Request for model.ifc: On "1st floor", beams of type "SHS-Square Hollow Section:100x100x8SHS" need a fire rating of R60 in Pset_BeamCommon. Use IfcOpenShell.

First a look at what the model holds.

```python
import ifcopenshell
import ifcopenshell.util.element

model = ifcopenshell.open("model.ifc")
print(model.schema)
storey = next(s for s in model.by_type("IfcBuildingStorey") if s.Name == "1st floor")
beams = [e for e in ifcopenshell.util.element.get_decomposition(storey) if e.is_a("IfcBeam")]
seen = {}
for e in beams:
    element_type = ifcopenshell.util.element.get_type(e)
    key = (element_type.Name if element_type != e and element_type else None, ifcopenshell.util.element.get_pset(e, "Pset_BeamCommon", "FireRating"))
    seen[key] = seen.get(key, 0) + 1
for (name, value), count in sorted(seen.items(), key=str):
    print(count, "x", name, "|", value)
```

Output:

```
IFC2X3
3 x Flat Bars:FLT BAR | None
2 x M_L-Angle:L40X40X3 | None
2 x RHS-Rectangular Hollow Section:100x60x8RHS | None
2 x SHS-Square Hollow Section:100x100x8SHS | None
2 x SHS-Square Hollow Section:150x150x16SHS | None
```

```python
import ifcopenshell
import ifcopenshell.api.pset
import ifcopenshell.util.element

model = ifcopenshell.open("model.ifc")

storey = next(s for s in model.by_type("IfcBuildingStorey") if s.Name == "1st floor")
beams = [e for e in ifcopenshell.util.element.get_decomposition(storey) if e.is_a("IfcBeam")]

count = 0
for e in beams:
    element_type = ifcopenshell.util.element.get_type(e)
    if element_type in (None, e) or element_type.Name != "SHS-Square Hollow Section:100x100x8SHS":
        continue
    # add_pset returns the element's existing set when there is one.
    pset = ifcopenshell.api.pset.add_pset(model, product=e, name="Pset_BeamCommon")
    ifcopenshell.api.pset.edit_pset(model, pset=pset, properties={"FireRating": "R60"})
    count += 1

print(count, "beams updated")

model.write("model_updated.ifc")
```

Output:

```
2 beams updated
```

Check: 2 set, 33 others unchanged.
